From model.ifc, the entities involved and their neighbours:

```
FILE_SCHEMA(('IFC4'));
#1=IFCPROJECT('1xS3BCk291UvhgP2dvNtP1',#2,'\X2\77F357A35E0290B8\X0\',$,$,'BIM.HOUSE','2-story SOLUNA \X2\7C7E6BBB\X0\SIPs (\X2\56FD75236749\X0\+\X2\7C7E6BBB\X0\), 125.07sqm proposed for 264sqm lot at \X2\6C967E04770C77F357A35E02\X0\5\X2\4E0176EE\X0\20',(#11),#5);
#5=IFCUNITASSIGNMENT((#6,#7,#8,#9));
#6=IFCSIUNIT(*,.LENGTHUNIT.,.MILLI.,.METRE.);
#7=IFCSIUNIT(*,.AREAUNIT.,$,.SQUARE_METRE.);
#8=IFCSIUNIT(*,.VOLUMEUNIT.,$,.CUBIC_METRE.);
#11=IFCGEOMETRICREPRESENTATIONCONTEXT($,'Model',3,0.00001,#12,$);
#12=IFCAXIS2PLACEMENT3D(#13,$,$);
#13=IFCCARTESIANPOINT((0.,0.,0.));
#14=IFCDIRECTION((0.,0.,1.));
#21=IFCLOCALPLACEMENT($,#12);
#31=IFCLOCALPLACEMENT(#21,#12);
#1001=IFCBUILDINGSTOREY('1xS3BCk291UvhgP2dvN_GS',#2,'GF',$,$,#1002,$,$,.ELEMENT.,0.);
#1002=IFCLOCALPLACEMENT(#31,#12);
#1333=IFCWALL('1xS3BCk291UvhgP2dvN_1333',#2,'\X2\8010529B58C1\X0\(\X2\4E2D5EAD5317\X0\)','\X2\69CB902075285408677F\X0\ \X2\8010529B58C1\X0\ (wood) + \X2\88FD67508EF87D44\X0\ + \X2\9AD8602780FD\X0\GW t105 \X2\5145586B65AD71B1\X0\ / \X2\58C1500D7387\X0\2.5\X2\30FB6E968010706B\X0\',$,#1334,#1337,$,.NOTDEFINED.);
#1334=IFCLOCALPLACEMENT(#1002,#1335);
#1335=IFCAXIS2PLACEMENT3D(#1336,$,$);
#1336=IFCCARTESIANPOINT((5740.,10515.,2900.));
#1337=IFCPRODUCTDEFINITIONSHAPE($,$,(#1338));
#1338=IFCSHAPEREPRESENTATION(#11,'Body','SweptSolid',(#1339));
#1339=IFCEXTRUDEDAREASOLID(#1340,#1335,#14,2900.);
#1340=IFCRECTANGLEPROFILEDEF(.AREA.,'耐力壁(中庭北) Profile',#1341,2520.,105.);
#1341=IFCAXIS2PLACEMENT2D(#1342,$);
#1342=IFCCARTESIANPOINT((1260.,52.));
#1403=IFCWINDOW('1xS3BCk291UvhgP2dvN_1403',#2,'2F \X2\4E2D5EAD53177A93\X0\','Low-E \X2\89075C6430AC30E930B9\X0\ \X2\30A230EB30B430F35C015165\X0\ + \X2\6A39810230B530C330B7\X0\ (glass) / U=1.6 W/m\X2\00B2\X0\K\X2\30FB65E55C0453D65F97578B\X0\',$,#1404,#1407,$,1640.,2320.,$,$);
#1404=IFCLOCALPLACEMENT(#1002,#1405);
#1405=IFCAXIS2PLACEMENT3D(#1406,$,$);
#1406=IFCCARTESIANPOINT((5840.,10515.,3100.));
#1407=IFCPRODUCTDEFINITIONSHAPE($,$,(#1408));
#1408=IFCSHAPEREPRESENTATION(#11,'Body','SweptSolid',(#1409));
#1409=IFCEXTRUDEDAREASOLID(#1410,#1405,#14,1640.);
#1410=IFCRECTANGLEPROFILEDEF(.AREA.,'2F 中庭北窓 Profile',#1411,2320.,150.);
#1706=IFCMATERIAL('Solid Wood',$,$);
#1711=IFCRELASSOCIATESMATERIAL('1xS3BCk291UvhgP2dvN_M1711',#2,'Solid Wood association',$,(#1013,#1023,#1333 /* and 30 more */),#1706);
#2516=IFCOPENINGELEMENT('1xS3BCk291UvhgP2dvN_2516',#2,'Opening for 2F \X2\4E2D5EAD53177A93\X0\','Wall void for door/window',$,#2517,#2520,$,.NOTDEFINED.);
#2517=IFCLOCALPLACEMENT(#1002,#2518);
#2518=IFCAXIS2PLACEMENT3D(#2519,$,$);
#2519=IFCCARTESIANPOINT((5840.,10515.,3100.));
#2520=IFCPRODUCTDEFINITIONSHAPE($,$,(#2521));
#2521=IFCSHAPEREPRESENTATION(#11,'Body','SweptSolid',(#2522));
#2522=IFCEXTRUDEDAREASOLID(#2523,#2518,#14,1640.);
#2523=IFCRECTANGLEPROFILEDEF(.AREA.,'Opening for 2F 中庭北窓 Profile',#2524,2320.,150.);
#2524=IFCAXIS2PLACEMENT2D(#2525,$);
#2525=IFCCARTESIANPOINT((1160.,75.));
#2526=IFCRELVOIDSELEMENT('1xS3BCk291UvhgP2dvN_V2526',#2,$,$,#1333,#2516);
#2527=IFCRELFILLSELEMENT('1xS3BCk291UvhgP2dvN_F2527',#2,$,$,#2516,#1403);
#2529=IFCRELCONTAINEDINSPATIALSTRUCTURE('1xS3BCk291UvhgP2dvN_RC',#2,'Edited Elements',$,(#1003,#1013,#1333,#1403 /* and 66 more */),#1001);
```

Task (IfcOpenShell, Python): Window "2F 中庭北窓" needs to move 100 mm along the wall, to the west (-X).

```python
import ifcopenshell
import ifcopenshell.api.geometry
import ifcopenshell.util.placement

model = ifcopenshell.open("model.ifc")

window = model.by_guid("1xS3BCk291UvhgP2dvN_1403")
opening = window.FillsVoids[0].RelatingOpeningElement
wall = opening.VoidsElements[0].RelatingBuildingElement

wall_matrix = ifcopenshell.util.placement.get_local_placement(wall.ObjectPlacement)
shift = wall_matrix[:3, 0] * -100.0
before = ifcopenshell.util.placement.get_local_placement(window.ObjectPlacement)[:3, 3].copy()

# The window is not placed relative to its opening, so move both.
for product in (opening, window):
    matrix = ifcopenshell.util.placement.get_local_placement(product.ObjectPlacement)
    matrix[:3, 3] += shift
    ifcopenshell.api.geometry.edit_object_placement(model, product=product, matrix=matrix, is_si=False)

after = ifcopenshell.util.placement.get_local_placement(window.ObjectPlacement)[:3, 3]
print("window moved by", (after - before).round(3) + 0.0)

model.write("model_updated.ifc")
```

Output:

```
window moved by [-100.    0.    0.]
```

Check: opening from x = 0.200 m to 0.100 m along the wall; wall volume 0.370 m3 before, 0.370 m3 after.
